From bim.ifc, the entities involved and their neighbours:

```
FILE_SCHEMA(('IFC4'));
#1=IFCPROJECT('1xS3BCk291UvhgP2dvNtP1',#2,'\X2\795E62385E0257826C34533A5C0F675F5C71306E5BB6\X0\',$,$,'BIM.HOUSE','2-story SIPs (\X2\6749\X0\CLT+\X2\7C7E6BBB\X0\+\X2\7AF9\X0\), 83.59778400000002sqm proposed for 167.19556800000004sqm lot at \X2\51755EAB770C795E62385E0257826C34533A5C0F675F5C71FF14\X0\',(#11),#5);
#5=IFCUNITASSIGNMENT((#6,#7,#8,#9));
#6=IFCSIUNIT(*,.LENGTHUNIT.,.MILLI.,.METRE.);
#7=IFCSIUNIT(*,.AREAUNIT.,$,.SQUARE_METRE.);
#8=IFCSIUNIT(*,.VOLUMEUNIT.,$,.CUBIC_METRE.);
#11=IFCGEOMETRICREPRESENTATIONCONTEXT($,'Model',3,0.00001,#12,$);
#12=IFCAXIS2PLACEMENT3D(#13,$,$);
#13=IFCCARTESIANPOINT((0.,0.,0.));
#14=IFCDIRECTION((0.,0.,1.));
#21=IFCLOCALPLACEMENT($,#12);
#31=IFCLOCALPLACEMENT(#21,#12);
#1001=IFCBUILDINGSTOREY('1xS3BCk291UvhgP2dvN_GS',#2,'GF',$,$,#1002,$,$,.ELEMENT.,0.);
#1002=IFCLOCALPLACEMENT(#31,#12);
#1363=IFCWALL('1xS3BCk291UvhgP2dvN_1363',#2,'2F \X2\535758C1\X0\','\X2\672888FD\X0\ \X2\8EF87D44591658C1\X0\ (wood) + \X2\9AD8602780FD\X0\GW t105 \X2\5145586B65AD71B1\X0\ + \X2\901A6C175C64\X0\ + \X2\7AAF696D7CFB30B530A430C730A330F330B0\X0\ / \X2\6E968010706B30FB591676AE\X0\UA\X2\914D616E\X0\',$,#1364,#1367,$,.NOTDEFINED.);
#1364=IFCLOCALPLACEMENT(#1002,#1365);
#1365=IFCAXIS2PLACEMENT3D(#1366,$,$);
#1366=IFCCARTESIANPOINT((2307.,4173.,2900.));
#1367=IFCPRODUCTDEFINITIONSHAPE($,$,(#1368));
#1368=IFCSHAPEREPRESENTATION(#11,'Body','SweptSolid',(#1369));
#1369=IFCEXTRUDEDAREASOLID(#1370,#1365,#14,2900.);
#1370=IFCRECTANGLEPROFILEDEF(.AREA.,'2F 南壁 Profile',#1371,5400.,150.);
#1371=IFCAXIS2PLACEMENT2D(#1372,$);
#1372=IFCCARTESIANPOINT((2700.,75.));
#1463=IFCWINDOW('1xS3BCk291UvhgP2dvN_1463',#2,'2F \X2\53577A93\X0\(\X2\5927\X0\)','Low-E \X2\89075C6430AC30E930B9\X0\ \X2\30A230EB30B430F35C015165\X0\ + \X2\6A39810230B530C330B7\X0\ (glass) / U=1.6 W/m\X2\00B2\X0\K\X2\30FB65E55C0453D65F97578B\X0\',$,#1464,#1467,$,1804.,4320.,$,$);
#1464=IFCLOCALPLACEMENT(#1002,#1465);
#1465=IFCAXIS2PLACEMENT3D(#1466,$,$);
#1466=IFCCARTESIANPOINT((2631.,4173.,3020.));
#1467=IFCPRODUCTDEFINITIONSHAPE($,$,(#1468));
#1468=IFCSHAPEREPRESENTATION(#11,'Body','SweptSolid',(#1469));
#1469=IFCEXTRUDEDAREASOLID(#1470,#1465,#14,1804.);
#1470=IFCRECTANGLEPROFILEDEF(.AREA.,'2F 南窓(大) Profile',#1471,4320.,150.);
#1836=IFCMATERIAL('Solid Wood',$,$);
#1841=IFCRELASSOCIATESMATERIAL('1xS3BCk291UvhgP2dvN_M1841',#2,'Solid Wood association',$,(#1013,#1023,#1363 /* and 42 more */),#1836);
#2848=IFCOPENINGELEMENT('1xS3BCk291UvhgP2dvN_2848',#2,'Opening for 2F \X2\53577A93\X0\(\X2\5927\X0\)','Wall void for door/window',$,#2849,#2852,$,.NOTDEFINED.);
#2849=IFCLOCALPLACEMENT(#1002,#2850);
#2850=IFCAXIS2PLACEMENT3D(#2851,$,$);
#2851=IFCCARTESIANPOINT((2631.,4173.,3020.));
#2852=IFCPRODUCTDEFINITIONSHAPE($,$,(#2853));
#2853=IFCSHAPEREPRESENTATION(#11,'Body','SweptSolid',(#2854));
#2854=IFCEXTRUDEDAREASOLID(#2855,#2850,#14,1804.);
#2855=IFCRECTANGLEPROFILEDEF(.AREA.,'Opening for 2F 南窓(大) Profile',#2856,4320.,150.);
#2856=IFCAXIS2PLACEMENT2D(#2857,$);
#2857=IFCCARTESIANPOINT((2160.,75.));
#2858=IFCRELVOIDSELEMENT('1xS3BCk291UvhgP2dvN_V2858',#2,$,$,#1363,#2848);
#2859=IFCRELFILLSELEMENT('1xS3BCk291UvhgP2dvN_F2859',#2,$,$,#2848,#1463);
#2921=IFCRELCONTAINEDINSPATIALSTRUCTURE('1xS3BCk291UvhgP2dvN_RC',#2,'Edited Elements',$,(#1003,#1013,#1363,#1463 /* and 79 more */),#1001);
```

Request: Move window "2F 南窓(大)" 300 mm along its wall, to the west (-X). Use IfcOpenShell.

```python
import ifcopenshell
import ifcopenshell.api.geometry
import ifcopenshell.util.placement
import ifcopenshell.util.unit

model = ifcopenshell.open("bim.ifc")
unit_scale = ifcopenshell.util.unit.calculate_unit_scale(model)

window = model.by_guid("1xS3BCk291UvhgP2dvN_1463")
opening = window.FillsVoids[0].RelatingOpeningElement
wall = opening.VoidsElements[0].RelatingBuildingElement

wall_matrix = ifcopenshell.util.placement.get_local_placement(wall.ObjectPlacement)
shift = wall_matrix[:3, 0] * -0.3 / unit_scale
before = ifcopenshell.util.placement.get_local_placement(window.ObjectPlacement)[:3, 3].copy()

# The window is not placed relative to its opening, so move both.
for product in (opening, window):
    matrix = ifcopenshell.util.placement.get_local_placement(product.ObjectPlacement)
    matrix[:3, 3] += shift
    ifcopenshell.api.geometry.edit_object_placement(model, product=product, matrix=matrix, is_si=False)

after = ifcopenshell.util.placement.get_local_placement(window.ObjectPlacement)[:3, 3]
print("window moved by", (after - before).round(3) + 0.0)

model.write("bim_edited.ifc")
```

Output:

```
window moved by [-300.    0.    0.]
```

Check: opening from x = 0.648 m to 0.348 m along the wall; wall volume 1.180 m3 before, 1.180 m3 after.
